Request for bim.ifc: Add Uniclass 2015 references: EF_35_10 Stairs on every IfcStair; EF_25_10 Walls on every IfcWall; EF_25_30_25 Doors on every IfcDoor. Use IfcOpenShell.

First a look at what the model holds.

```python
import ifcopenshell

model = ifcopenshell.open("bim.ifc")
print(model.schema)
print("classifications:", [c.Name for c in model.by_type("IfcClassification")])
for ifc_class in ("IfcDoor", "IfcRoof", "IfcStair", "IfcWall", "IfcWindow"):
    print(ifc_class, len(model.by_type(ifc_class)))
```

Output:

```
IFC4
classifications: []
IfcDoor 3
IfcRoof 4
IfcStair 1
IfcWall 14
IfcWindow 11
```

```python
import ifcopenshell
import ifcopenshell.api.classification

model = ifcopenshell.open("bim.ifc")

system = ifcopenshell.api.classification.add_classification(model, classification="Uniclass 2015")

codes = {
    "IfcStair": ("EF_35_10", "Stairs"),
    "IfcWall": ("EF_25_10", "Walls"),
    "IfcDoor": ("EF_25_30_25", "Doors"),
}
for ifc_class, (code, name) in codes.items():
    products = model.by_type(ifc_class)
    ifcopenshell.api.classification.add_reference(
        model, products=products, classification=system, identification=code, name=name
    )
    print(code, len(products))

model.write("bim_v2.ifc")
```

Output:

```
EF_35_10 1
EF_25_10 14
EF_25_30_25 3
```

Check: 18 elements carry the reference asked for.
